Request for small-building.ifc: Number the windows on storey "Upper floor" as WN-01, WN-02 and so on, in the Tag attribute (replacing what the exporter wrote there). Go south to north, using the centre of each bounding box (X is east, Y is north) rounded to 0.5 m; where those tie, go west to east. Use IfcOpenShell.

First a look at what the model holds.

```python
import ifcopenshell
import ifcopenshell.util.element
import ifcopenshell.util.placement

model = ifcopenshell.open("small-building.ifc")
print(model.schema)
storey = next(s for s in model.by_type("IfcBuildingStorey") if s.Name == "Upper floor")
windows = [e for e in ifcopenshell.util.element.get_decomposition(storey) if e.is_a("IfcWindow")]
for e in sorted(windows, key=lambda e: e.id()):
    origin = ifcopenshell.util.placement.get_local_placement(e.ObjectPlacement)[:3, 3]
    print(e.id(), e.Tag, e.Name, origin.round(2) + 0.0, sep=" | ")
```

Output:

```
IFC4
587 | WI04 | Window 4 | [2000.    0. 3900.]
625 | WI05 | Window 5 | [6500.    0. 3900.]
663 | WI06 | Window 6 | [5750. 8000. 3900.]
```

```python
import ifcopenshell
import ifcopenshell.geom
import ifcopenshell.util.element
import ifcopenshell.util.shape

model = ifcopenshell.open("small-building.ifc")
settings = ifcopenshell.geom.settings()
settings.set("use-world-coords", True)


def centre(element):
    shape = ifcopenshell.geom.create_shape(settings, element)
    return ifcopenshell.util.shape.get_bbox_centroid(shape.geometry)


storey = next(s for s in model.by_type("IfcBuildingStorey") if s.Name == "Upper floor")
windows = [e for e in ifcopenshell.util.element.get_decomposition(storey) if e.is_a("IfcWindow")]

# Insertion points can sit at a corner or the storey origin, so sort by the geometry (in metres).
centres = {e: centre(e) for e in windows}
windows.sort(key=lambda e: (round(centres[e][1] / 0.5), centres[e][0]))

for i, e in enumerate(windows, start=1):
    number = f"WN-{i:02d}"
    e.Tag = number
    print(e.id(), number)

model.write("small-building_edited.ifc")
```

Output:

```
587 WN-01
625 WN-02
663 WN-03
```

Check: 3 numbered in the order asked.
